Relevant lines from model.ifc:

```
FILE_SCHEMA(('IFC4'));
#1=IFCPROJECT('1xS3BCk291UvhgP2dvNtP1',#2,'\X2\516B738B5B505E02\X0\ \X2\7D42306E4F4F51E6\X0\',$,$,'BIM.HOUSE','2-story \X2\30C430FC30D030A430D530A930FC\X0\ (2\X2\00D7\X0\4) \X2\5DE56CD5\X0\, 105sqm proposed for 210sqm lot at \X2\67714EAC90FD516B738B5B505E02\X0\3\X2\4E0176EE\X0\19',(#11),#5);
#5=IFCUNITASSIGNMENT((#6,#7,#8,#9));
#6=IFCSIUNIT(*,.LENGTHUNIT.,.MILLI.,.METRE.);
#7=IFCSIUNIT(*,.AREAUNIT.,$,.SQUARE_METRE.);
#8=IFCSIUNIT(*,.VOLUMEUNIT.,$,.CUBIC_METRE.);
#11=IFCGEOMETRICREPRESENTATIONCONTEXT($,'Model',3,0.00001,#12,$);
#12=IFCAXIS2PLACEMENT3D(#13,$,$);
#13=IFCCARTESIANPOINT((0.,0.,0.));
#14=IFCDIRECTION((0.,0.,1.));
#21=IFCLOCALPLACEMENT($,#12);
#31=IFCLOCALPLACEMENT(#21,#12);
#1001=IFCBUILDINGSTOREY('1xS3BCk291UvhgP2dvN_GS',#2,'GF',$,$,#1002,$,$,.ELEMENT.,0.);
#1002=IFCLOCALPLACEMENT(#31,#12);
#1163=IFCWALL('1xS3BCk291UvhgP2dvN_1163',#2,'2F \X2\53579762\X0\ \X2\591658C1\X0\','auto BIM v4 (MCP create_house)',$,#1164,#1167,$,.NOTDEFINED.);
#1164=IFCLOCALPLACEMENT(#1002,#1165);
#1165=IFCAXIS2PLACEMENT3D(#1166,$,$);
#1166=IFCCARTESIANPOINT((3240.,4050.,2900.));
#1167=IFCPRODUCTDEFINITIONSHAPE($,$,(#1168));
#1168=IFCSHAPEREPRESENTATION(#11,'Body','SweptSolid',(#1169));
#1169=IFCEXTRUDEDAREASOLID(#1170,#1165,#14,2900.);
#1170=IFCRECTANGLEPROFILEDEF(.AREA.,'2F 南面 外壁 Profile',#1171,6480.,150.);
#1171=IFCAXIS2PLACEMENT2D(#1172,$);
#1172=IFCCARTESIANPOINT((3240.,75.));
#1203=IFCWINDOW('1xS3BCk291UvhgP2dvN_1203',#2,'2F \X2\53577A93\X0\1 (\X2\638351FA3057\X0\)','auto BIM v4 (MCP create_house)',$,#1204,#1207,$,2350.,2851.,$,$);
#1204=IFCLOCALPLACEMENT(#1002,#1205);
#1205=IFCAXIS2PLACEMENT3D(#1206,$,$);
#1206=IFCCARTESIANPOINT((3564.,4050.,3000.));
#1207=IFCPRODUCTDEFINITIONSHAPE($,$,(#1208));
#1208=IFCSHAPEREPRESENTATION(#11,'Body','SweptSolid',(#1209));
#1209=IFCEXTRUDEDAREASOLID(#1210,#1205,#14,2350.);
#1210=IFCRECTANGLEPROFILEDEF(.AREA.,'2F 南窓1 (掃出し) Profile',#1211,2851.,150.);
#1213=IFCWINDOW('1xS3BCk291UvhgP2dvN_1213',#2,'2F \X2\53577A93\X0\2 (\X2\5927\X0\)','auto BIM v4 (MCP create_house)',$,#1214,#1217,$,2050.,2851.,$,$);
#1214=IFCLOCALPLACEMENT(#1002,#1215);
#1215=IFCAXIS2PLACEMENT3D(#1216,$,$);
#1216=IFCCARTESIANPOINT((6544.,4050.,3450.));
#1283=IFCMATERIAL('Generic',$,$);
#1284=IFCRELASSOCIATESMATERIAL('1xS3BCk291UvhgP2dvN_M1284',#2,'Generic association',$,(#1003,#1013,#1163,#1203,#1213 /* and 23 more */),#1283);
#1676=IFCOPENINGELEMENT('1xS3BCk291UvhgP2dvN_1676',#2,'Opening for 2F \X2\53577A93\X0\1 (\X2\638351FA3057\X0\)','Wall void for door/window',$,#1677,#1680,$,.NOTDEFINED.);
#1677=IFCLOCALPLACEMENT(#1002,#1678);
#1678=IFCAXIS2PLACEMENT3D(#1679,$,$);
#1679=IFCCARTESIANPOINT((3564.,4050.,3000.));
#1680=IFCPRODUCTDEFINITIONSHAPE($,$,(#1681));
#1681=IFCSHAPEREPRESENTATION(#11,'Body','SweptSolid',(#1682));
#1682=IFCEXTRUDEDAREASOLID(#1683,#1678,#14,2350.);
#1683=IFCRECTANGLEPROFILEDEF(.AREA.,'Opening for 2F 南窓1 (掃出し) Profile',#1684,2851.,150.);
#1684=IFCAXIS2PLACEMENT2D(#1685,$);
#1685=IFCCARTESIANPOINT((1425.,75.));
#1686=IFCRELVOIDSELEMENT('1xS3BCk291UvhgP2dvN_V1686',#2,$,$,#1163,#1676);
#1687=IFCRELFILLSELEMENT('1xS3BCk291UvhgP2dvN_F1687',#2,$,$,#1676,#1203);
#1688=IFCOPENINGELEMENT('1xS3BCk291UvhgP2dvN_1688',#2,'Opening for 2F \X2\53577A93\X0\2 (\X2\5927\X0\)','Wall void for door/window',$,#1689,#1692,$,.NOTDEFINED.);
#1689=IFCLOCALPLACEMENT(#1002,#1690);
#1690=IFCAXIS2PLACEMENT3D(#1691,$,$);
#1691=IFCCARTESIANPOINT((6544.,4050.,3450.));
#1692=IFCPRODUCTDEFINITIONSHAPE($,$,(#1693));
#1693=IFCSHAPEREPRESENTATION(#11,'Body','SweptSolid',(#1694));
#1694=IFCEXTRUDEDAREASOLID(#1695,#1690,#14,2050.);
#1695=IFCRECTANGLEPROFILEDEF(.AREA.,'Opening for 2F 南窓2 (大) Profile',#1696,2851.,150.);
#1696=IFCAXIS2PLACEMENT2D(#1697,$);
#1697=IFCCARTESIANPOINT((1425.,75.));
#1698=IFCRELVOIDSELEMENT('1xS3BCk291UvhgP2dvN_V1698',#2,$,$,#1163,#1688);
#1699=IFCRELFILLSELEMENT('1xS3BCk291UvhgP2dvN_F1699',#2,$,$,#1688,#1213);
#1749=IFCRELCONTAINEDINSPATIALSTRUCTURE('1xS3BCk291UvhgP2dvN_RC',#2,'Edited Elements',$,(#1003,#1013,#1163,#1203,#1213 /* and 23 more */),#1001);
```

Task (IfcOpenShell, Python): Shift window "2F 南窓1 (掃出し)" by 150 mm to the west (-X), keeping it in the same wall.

```python
import ifcopenshell
import ifcopenshell.api.geometry
import ifcopenshell.util.placement

model = ifcopenshell.open("model.ifc")

window = model.by_guid("1xS3BCk291UvhgP2dvN_1203")
opening = window.FillsVoids[0].RelatingOpeningElement
wall = opening.VoidsElements[0].RelatingBuildingElement

wall_matrix = ifcopenshell.util.placement.get_local_placement(wall.ObjectPlacement)
shift = wall_matrix[:3, 0] * -150.0
before = ifcopenshell.util.placement.get_local_placement(window.ObjectPlacement)[:3, 3].copy()

# The window is not placed relative to its opening, so move both.
for product in (opening, window):
    matrix = ifcopenshell.util.placement.get_local_placement(product.ObjectPlacement)
    matrix[:3, 3] += shift
    ifcopenshell.api.geometry.edit_object_placement(model, product=product, matrix=matrix, is_si=False)

after = ifcopenshell.util.placement.get_local_placement(window.ObjectPlacement)[:3, 3]
print("window moved by", (after - before).round(3) + 0.0)

model.write("model-out.ifc")
```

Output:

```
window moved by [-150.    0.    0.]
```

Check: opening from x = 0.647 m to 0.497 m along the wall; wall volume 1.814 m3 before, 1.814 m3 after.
